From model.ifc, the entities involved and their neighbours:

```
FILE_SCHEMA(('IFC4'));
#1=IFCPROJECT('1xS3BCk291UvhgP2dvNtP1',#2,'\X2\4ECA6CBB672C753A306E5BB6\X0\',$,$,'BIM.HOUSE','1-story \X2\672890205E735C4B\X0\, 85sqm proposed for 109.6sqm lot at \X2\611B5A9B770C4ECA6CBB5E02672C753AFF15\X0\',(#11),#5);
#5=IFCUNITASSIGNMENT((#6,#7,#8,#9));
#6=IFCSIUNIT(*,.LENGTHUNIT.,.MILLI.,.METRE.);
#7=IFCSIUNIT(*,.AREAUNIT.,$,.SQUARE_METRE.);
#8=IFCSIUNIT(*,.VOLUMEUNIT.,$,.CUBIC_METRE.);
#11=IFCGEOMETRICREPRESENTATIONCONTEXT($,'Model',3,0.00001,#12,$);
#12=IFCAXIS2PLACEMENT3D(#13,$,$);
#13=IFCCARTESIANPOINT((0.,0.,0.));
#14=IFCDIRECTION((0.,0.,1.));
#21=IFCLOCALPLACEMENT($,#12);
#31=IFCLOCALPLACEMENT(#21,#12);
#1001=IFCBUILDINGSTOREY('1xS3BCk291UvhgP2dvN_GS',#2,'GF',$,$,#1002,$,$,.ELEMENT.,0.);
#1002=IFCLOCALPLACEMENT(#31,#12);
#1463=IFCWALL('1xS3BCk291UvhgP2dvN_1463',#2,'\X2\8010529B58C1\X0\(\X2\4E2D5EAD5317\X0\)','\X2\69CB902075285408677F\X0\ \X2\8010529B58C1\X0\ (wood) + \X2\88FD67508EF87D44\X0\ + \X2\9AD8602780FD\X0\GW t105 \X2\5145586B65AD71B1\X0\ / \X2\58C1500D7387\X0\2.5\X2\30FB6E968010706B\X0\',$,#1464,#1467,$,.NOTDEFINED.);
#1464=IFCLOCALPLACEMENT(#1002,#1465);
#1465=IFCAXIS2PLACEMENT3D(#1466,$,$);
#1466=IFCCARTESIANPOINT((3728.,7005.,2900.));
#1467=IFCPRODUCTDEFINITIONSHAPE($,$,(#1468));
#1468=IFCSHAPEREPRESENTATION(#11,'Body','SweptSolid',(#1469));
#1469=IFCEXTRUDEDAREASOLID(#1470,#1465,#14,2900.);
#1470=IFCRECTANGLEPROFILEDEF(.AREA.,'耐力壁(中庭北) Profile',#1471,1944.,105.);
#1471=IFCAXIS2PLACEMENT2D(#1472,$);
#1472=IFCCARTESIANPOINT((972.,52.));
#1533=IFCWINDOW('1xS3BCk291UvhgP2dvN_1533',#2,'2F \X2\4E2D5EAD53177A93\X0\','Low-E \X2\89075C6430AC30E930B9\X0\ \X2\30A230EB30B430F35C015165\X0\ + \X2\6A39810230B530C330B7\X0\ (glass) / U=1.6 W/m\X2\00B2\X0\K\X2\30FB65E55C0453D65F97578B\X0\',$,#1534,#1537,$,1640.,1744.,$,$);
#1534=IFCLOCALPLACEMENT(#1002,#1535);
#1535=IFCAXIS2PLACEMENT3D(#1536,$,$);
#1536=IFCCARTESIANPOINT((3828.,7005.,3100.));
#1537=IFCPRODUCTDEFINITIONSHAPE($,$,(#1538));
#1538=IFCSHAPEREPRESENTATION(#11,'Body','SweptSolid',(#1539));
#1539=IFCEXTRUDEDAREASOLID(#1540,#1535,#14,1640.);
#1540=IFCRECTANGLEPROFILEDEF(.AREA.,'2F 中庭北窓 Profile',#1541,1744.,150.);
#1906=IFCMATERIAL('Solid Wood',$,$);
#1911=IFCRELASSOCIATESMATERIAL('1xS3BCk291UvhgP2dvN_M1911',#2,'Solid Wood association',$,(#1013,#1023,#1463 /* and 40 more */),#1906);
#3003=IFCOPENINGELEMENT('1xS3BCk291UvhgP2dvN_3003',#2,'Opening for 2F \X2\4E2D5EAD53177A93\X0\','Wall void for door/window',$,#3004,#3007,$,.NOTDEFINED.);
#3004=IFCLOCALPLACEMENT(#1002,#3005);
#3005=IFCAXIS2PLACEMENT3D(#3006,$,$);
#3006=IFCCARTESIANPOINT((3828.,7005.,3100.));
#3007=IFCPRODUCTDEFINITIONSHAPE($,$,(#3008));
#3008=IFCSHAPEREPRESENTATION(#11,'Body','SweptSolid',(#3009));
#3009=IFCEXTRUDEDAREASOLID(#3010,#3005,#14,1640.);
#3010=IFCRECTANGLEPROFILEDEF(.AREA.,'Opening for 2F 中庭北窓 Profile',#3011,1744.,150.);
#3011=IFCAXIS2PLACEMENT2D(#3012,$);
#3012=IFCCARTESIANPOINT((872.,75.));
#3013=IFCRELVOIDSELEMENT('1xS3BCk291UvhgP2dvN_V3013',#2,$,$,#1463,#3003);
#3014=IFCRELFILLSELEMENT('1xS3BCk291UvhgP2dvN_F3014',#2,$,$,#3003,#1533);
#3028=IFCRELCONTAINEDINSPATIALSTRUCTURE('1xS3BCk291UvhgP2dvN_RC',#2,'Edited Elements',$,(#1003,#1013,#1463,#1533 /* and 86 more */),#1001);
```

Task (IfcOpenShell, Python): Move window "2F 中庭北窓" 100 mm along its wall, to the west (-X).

```python
import ifcopenshell
import ifcopenshell.api.geometry
import ifcopenshell.util.placement
import ifcopenshell.util.unit

model = ifcopenshell.open("model.ifc")
unit_scale = ifcopenshell.util.unit.calculate_unit_scale(model)

window = model.by_guid("1xS3BCk291UvhgP2dvN_1533")
opening = window.FillsVoids[0].RelatingOpeningElement
wall = opening.VoidsElements[0].RelatingBuildingElement

wall_matrix = ifcopenshell.util.placement.get_local_placement(wall.ObjectPlacement)
shift = wall_matrix[:3, 0] * -0.1 / unit_scale
before = ifcopenshell.util.placement.get_local_placement(window.ObjectPlacement)[:3, 3].copy()

# The window is not placed relative to its opening, so move both.
for product in (opening, window):
    matrix = ifcopenshell.util.placement.get_local_placement(product.ObjectPlacement)
    matrix[:3, 3] += shift
    ifcopenshell.api.geometry.edit_object_placement(model, product=product, matrix=matrix, is_si=False)

after = ifcopenshell.util.placement.get_local_placement(window.ObjectPlacement)[:3, 3]
print("window moved by", (after - before).round(3) + 0.0)

model.write("model-out.ifc")
```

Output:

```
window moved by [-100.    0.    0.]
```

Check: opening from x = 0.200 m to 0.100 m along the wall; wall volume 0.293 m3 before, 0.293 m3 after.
